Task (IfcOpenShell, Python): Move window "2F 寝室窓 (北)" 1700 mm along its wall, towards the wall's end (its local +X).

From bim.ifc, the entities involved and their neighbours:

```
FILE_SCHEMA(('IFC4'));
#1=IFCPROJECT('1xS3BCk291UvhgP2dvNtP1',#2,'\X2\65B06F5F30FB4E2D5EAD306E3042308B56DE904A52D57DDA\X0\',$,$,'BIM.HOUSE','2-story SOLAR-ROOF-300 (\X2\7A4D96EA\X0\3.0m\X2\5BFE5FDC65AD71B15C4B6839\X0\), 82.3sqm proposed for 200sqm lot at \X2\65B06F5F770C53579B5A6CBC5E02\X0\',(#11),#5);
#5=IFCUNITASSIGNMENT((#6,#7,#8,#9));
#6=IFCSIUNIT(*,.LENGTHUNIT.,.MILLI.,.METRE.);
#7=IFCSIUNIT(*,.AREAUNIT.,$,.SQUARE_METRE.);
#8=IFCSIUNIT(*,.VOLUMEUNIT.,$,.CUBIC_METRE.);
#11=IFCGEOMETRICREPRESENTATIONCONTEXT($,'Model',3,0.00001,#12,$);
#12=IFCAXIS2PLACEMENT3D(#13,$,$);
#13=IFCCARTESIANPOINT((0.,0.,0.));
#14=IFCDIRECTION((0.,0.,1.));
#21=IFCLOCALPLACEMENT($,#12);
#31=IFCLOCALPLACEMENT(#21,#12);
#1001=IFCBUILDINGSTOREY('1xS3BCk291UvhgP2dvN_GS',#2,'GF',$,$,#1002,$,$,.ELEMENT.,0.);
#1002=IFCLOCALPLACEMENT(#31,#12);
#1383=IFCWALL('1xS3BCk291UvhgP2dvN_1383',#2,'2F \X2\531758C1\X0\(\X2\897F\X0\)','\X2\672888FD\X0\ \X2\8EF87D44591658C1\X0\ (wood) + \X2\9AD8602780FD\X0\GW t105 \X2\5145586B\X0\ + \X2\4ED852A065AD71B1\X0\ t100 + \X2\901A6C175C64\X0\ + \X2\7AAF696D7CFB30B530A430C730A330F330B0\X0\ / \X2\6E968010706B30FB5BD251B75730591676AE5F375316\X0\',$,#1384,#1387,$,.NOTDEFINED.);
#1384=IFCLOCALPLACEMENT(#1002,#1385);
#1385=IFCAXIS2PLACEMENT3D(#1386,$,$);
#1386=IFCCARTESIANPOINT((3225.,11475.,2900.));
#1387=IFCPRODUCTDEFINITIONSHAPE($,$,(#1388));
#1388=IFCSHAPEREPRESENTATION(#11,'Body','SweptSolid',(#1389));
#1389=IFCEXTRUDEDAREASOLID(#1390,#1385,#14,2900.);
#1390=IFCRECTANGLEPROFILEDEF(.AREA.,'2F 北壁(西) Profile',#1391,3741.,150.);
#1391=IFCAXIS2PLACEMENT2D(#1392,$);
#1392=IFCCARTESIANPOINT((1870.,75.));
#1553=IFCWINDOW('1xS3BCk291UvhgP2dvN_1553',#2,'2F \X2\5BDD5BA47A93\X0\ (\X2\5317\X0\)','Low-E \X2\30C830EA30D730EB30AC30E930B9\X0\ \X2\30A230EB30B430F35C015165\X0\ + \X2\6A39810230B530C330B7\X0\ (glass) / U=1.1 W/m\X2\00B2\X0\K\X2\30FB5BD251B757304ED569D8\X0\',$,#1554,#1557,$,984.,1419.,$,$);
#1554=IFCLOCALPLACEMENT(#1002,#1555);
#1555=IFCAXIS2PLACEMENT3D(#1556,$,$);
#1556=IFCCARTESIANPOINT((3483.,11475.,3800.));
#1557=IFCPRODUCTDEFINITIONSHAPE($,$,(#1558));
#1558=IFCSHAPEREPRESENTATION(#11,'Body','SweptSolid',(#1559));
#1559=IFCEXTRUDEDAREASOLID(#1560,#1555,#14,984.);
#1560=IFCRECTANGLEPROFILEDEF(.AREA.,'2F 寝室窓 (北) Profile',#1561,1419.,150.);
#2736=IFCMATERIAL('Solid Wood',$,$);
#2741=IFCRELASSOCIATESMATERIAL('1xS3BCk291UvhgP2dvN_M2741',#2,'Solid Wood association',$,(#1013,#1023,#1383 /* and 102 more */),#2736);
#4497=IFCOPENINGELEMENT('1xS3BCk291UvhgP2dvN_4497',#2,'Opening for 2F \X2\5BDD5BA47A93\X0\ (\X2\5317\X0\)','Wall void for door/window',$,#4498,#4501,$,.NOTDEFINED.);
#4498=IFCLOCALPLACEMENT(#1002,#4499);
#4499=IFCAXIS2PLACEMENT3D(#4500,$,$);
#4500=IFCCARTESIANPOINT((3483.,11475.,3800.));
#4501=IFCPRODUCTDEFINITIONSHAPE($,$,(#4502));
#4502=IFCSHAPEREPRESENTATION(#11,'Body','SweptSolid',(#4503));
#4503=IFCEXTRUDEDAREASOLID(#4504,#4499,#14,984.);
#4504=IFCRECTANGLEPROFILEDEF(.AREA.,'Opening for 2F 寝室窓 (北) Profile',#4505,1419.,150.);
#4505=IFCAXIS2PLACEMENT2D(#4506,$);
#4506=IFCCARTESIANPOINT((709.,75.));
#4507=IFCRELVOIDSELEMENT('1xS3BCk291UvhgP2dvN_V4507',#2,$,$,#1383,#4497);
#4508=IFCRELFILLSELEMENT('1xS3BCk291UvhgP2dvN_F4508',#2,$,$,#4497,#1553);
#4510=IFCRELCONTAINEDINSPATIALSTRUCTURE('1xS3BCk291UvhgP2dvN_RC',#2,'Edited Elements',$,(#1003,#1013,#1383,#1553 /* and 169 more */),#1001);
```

```python
import ifcopenshell
import ifcopenshell.api.geometry
import ifcopenshell.util.placement

model = ifcopenshell.open("bim.ifc")

window = model.by_guid("1xS3BCk291UvhgP2dvN_1553")
opening = window.FillsVoids[0].RelatingOpeningElement
wall = opening.VoidsElements[0].RelatingBuildingElement

wall_matrix = ifcopenshell.util.placement.get_local_placement(wall.ObjectPlacement)
shift = wall_matrix[:3, 0] * 1700.0
before = ifcopenshell.util.placement.get_local_placement(window.ObjectPlacement)[:3, 3].copy()

# The window is not placed relative to its opening, so move both.
for product in (opening, window):
    matrix = ifcopenshell.util.placement.get_local_placement(product.ObjectPlacement)
    matrix[:3, 3] += shift
    ifcopenshell.api.geometry.edit_object_placement(model, product=product, matrix=matrix, is_si=False)

after = ifcopenshell.util.placement.get_local_placement(window.ObjectPlacement)[:3, 3]
print("window moved by", (after - before).round(3) + 0.0)

model.write("bim_rev.ifc")
```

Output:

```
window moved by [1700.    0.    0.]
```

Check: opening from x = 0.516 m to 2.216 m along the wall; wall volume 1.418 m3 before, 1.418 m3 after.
